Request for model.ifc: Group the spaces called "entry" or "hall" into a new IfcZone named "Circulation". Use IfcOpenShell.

First a look at what the model holds.

```python
import ifcopenshell

model = ifcopenshell.open("model.ifc")
print(model.schema)
seen = {}
for space in model.by_type("IfcSpace"):
    seen[space.LongName] = seen.get(space.LongName, 0) + 1
for name, count in sorted(seen.items(), key=str):
    print(count, "x", name)
print("zones:", [z.Name for z in model.by_type("IfcZone")][:20])
```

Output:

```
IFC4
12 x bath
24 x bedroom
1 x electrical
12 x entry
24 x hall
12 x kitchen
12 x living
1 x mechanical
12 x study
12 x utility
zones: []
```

```python
import ifcopenshell
import ifcopenshell.api.group
import ifcopenshell.api.root

model = ifcopenshell.open("model.ifc")

names = {"entry", "hall"}
spaces = [s for s in model.by_type("IfcSpace") if s.LongName in names]

zone = ifcopenshell.api.root.create_entity(model, ifc_class="IfcZone", name="Circulation")
ifcopenshell.api.group.assign_group(model, products=spaces, group=zone)
print(len(spaces), "spaces in", zone.Name)

model.write("model-out.ifc")
```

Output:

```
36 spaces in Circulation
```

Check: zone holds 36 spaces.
